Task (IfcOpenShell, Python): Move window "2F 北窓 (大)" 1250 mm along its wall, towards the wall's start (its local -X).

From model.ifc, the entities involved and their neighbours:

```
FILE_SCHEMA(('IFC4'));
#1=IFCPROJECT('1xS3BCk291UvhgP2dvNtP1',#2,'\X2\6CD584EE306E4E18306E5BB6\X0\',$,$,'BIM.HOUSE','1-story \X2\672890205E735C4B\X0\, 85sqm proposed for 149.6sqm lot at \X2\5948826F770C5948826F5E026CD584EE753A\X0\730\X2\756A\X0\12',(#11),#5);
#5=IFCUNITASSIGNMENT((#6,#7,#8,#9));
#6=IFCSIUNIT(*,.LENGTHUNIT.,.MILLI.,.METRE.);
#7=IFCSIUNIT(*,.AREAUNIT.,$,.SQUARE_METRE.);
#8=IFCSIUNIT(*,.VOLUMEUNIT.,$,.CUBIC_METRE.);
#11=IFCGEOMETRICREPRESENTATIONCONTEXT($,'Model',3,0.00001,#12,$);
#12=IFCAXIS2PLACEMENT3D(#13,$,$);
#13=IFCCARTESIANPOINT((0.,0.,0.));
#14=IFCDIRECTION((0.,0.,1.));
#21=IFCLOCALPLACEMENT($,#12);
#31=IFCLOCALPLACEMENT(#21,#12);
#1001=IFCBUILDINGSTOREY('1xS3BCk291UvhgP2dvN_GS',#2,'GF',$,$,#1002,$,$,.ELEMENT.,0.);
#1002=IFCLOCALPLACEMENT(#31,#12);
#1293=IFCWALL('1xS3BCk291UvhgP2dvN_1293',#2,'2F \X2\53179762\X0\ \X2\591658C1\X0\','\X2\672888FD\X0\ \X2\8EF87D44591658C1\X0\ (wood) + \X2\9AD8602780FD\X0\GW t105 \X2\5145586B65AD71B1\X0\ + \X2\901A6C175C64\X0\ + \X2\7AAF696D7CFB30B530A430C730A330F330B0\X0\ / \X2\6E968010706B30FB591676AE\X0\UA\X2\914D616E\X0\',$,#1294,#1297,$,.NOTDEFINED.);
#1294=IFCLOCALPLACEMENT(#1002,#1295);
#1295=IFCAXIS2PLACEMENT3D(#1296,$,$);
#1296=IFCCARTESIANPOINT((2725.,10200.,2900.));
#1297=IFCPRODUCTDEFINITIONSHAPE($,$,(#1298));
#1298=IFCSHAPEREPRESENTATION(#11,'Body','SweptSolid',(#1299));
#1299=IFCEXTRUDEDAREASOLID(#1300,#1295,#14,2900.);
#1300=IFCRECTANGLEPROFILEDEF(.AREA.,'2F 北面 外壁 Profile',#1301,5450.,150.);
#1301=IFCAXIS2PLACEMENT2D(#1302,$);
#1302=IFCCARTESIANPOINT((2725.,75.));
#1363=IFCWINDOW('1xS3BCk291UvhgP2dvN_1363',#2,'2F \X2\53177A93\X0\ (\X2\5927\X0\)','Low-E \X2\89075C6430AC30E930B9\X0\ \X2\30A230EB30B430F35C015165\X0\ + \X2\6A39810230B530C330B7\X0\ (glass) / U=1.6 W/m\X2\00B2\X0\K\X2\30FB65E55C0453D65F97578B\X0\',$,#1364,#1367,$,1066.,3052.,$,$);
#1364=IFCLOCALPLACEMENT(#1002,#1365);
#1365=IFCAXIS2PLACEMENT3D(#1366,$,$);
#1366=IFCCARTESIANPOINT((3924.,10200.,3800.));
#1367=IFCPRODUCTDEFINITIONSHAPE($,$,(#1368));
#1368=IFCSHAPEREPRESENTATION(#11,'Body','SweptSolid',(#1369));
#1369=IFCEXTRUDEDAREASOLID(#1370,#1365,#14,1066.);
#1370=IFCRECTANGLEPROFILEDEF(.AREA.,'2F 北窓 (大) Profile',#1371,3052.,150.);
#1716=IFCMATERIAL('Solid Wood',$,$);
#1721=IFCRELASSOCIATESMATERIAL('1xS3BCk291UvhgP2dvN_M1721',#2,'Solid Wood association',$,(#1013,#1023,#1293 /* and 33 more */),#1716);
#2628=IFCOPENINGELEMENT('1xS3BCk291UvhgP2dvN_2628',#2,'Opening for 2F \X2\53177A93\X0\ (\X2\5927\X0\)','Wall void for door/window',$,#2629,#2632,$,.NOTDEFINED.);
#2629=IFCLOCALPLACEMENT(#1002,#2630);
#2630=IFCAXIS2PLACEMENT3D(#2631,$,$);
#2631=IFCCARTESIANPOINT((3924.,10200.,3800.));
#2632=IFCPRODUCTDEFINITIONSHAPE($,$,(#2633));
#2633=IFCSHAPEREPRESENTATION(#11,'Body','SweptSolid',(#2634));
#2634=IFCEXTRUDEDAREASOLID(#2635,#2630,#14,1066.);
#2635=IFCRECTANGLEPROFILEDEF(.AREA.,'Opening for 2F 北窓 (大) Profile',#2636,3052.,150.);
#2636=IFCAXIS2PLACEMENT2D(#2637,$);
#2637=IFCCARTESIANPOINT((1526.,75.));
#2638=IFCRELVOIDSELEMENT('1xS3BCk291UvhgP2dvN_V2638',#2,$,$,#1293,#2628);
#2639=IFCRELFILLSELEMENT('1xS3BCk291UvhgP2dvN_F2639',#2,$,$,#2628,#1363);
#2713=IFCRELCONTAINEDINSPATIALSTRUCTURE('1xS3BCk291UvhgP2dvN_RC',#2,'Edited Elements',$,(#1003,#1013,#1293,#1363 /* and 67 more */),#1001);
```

```python
import ifcopenshell
import ifcopenshell.api.geometry
import ifcopenshell.util.placement
import ifcopenshell.util.unit

model = ifcopenshell.open("model.ifc")
unit_scale = ifcopenshell.util.unit.calculate_unit_scale(model)

window = model.by_guid("1xS3BCk291UvhgP2dvN_1363")
opening = window.FillsVoids[0].RelatingOpeningElement
wall = opening.VoidsElements[0].RelatingBuildingElement

wall_matrix = ifcopenshell.util.placement.get_local_placement(wall.ObjectPlacement)
shift = wall_matrix[:3, 0] * -1.25 / unit_scale
before = ifcopenshell.util.placement.get_local_placement(window.ObjectPlacement)[:3, 3].copy()

# The window is not placed relative to its opening, so move both.
for product in (opening, window):
    matrix = ifcopenshell.util.placement.get_local_placement(product.ObjectPlacement)
    matrix[:3, 3] += shift
    ifcopenshell.api.geometry.edit_object_placement(model, product=product, matrix=matrix, is_si=False)

after = ifcopenshell.util.placement.get_local_placement(window.ObjectPlacement)[:3, 3]
print("window moved by", (after - before).round(3) + 0.0)

model.write("model_edited.ifc")
```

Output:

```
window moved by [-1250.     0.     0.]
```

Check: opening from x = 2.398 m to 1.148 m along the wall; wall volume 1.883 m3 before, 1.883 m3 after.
